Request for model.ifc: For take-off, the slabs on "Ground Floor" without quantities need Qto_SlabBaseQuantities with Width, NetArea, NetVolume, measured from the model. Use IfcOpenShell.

First a look at what the model holds.

```python
import ifcopenshell
import ifcopenshell.util.element
import ifcopenshell.util.unit

model = ifcopenshell.open("model.ifc")
print(model.schema)
for unit_type in ("LENGTHUNIT", "AREAUNIT", "VOLUMEUNIT"):
    print(unit_type, ifcopenshell.util.unit.calculate_unit_scale(model, unit_type))
storey = next(s for s in model.by_type("IfcBuildingStorey") if s.Name == "Ground Floor")
slabs = [e for e in ifcopenshell.util.element.get_decomposition(storey) if e.is_a("IfcSlab")]
for e in sorted(slabs, key=lambda e: e.id()):
    print(e.id(), e.is_a(), e.Name, list(ifcopenshell.util.element.get_psets(e, qtos_only=True)), sep=" | ")
```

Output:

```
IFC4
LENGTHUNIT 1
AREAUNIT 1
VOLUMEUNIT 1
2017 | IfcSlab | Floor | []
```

```python
import ifcopenshell
import ifcopenshell.api.pset
import ifcopenshell.geom
import ifcopenshell.util.element
import ifcopenshell.util.shape
import ifcopenshell.util.unit

model = ifcopenshell.open("model.ifc")
unit_scale = ifcopenshell.util.unit.calculate_unit_scale(model)
area_scale = ifcopenshell.util.unit.calculate_unit_scale(model, "AREAUNIT")
volume_scale = ifcopenshell.util.unit.calculate_unit_scale(model, "VOLUMEUNIT")
settings = ifcopenshell.geom.settings()

storey = next(s for s in model.by_type("IfcBuildingStorey") if s.Name == "Ground Floor")
slabs = [e for e in ifcopenshell.util.element.get_decomposition(storey) if e.is_a("IfcSlab")]

for e in sorted(slabs, key=lambda e: e.id()):
    if ifcopenshell.util.element.get_psets(e, qtos_only=True, should_inherit=False):
        continue
    # Geometry comes back in metres, in the element's own axes.
    shape = ifcopenshell.geom.create_shape(settings, e)
    values = {
        "Width": ifcopenshell.util.shape.get_z(shape.geometry) / unit_scale,
        "NetArea": ifcopenshell.util.shape.get_footprint_area(shape.geometry) / area_scale,
        "NetVolume": ifcopenshell.util.shape.get_volume(shape.geometry) / volume_scale,
    }
    qto = ifcopenshell.api.pset.add_qto(model, product=e, name="Qto_SlabBaseQuantities")
    ifcopenshell.api.pset.edit_qto(model, qto=qto, properties=values)
    print(e.id(), {k: round(v, 3) for k, v in values.items()})

model.write("model_edited.ifc")
```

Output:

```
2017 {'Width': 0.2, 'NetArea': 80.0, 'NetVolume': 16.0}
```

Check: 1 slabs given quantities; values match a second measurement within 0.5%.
